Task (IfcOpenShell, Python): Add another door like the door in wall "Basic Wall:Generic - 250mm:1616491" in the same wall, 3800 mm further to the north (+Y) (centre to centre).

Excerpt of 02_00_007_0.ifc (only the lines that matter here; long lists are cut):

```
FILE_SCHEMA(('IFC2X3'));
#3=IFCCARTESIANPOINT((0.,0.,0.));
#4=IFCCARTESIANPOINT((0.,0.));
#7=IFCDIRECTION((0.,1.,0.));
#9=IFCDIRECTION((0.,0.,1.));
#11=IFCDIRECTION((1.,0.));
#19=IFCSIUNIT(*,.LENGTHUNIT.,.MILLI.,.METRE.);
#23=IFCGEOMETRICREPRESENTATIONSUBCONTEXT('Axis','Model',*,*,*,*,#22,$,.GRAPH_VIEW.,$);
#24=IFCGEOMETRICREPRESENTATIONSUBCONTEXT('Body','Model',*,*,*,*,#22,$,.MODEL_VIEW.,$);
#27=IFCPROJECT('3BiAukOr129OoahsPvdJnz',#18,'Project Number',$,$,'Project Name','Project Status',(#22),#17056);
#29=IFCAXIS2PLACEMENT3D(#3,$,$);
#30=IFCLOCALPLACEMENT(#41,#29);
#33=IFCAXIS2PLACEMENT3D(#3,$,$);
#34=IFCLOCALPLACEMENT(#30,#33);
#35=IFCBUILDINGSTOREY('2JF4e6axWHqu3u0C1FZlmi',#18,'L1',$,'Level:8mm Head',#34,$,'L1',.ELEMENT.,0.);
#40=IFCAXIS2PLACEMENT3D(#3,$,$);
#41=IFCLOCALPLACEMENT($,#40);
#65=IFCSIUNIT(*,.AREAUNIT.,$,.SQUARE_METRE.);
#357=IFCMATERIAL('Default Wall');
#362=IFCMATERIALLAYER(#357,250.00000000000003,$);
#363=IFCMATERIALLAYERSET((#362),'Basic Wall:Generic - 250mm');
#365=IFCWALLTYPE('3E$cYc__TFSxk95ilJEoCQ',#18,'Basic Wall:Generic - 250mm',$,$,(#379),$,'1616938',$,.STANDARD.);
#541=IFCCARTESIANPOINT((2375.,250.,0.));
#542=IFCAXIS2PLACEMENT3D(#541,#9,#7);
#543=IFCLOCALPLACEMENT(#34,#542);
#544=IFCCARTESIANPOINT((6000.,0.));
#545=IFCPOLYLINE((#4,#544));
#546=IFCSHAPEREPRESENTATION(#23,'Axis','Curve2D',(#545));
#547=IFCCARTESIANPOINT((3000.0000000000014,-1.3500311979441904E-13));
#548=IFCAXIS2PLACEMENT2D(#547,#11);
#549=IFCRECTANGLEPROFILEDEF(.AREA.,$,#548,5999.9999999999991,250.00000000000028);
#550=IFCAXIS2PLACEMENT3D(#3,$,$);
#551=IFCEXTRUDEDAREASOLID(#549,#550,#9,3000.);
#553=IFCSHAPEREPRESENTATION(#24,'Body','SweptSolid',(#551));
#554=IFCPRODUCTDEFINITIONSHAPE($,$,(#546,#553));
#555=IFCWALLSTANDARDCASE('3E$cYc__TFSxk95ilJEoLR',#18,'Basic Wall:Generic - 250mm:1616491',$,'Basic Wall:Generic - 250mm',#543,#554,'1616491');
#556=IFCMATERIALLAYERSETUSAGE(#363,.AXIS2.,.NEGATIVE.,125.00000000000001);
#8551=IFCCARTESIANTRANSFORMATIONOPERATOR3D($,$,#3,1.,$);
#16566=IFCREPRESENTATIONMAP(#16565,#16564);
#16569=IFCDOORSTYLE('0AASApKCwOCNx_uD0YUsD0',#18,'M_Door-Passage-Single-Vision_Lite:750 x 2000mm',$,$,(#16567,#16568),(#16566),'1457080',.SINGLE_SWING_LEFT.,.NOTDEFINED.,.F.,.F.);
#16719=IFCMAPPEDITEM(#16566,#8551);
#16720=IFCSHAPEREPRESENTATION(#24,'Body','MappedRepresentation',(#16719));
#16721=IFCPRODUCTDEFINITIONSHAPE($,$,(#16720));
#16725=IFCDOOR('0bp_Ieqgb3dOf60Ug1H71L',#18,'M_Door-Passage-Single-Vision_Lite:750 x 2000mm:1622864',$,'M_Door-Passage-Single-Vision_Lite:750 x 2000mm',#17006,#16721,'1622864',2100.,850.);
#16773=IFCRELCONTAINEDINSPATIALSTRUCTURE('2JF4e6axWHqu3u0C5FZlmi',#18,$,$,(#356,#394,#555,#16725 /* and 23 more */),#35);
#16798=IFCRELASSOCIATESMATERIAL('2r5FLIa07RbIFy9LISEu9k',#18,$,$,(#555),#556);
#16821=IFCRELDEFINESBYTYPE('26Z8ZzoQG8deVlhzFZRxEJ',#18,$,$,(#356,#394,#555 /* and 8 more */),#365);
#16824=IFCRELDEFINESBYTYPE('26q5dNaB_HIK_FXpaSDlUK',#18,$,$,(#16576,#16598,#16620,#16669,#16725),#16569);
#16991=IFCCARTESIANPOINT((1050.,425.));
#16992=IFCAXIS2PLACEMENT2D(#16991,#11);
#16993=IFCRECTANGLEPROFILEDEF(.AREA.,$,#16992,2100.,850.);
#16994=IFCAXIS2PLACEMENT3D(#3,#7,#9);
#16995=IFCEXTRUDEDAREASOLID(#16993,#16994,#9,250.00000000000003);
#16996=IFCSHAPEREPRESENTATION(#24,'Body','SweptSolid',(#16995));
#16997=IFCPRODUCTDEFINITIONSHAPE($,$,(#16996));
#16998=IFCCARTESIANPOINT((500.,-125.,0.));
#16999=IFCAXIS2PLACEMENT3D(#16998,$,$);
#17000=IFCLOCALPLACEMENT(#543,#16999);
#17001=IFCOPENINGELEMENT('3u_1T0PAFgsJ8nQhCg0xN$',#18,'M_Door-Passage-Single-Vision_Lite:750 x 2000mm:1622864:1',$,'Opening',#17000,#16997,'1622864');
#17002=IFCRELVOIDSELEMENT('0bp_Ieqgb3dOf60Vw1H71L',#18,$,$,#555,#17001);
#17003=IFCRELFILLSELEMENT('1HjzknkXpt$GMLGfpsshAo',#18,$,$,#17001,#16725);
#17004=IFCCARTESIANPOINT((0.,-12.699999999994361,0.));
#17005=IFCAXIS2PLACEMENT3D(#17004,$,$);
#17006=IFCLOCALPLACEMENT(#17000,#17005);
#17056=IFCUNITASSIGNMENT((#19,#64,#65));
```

```python
import ifcopenshell
import ifcopenshell.api.feature
import ifcopenshell.api.geometry
import ifcopenshell.api.root
import ifcopenshell.geom
import ifcopenshell.util.element
import ifcopenshell.util.placement
import ifcopenshell.util.shape

model = ifcopenshell.open("02_00_007_0.ifc")
settings = ifcopenshell.geom.settings()


def volume(element):
    """Net volume in cubic metres, openings subtracted."""
    shape = ifcopenshell.geom.create_shape(settings, element)
    return ifcopenshell.util.shape.get_volume(shape.geometry)


def reuse_history(source, copy):
    """copy_class also copies each property set's owner history, people and application; keep the originals."""
    for rel in copy.IsDefinedBy:
        if rel.is_a("IfcRelDefinesByProperties") and (history := rel.RelatingPropertyDefinition.OwnerHistory):
            rel.RelatingPropertyDefinition.OwnerHistory = source.OwnerHistory
            ifcopenshell.util.element.remove_deep2(model, history)


door = model.by_guid("0bp_Ieqgb3dOf60Ug1H71L")
opening = door.FillsVoids[0].RelatingOpeningElement
wall = opening.VoidsElements[0].RelatingBuildingElement
before = volume(wall)
shift = ifcopenshell.util.placement.get_local_placement(wall.ObjectPlacement)[:3, 0] * 3800.0

# copy_class copies the void relationship, type, container and properties, but no geometry.
new_opening = ifcopenshell.api.root.copy_class(model, product=opening)
new_opening.Representation = ifcopenshell.util.element.copy_deep(
    model, opening.Representation, exclude=["IfcGeometricRepresentationContext", "IfcRepresentationMap"]
)
new_opening.Name = "M_Door-Passage-Single-Vision_Lite:750 x 2000mm"
new_opening.Tag = None
new_door = ifcopenshell.api.root.copy_class(model, product=door)
new_door.Representation = ifcopenshell.util.element.copy_deep(
    model, door.Representation, exclude=["IfcGeometricRepresentationContext", "IfcRepresentationMap"]
)
new_door.Name = "M_Door-Passage-Single-Vision_Lite:750 x 2000mm"
new_door.Tag = None
reuse_history(door, new_door)
fills = ifcopenshell.api.feature.add_filling(model, opening=new_opening, element=new_door)
fills.OwnerHistory = new_door.OwnerHistory  # required in IFC2X3

for old, new in ((opening, new_opening), (door, new_door)):
    matrix = ifcopenshell.util.placement.get_local_placement(old.ObjectPlacement)
    matrix[:3, 3] += shift
    ifcopenshell.api.geometry.edit_object_placement(model, product=new, matrix=matrix, is_si=False)

after = volume(wall)

print(f"wall volume {before:.3f} -> {after:.3f} m3")

model.write("02_00_007_0-out.ifc")
```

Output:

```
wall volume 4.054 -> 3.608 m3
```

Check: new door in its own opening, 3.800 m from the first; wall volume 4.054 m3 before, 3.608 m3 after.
